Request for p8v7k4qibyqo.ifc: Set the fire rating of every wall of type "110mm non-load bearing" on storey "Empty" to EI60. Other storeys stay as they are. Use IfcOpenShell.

First a look at what the model holds.

```python
import ifcopenshell
import ifcopenshell.util.element

model = ifcopenshell.open("p8v7k4qibyqo.ifc")
print(model.schema)
storey = next(s for s in model.by_type("IfcBuildingStorey") if s.Name == "Empty")
walls = [e for e in ifcopenshell.util.element.get_decomposition(storey) if e.is_a("IfcWall")]
seen = {}
for e in walls:
    element_type = ifcopenshell.util.element.get_type(e)
    key = (element_type.Name if element_type != e and element_type else None, ifcopenshell.util.element.get_pset(e, "Pset_WallCommon", "FireRating"))
    seen[key] = seen.get(key, 0) + 1
for (name, value), count in sorted(seen.items(), key=str):
    print(count, "x", name, "|", value)
```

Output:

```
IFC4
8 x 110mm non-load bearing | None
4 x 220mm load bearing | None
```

```python
import ifcopenshell
import ifcopenshell.api.pset
import ifcopenshell.util.element

model = ifcopenshell.open("p8v7k4qibyqo.ifc")

storey = next(s for s in model.by_type("IfcBuildingStorey") if s.Name == "Empty")
walls = [e for e in ifcopenshell.util.element.get_decomposition(storey) if e.is_a("IfcWall")]

count = 0
for e in walls:
    element_type = ifcopenshell.util.element.get_type(e)
    if element_type in (None, e) or element_type.Name != "110mm non-load bearing":
        continue
    # add_pset returns the element's existing set when there is one.
    pset = ifcopenshell.api.pset.add_pset(model, product=e, name="Pset_WallCommon")
    ifcopenshell.api.pset.edit_pset(model, pset=pset, properties={"FireRating": "EI60"})
    count += 1

print(count, "walls updated")

model.write("p8v7k4qibyqo_updated.ifc")
```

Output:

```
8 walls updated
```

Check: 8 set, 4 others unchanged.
